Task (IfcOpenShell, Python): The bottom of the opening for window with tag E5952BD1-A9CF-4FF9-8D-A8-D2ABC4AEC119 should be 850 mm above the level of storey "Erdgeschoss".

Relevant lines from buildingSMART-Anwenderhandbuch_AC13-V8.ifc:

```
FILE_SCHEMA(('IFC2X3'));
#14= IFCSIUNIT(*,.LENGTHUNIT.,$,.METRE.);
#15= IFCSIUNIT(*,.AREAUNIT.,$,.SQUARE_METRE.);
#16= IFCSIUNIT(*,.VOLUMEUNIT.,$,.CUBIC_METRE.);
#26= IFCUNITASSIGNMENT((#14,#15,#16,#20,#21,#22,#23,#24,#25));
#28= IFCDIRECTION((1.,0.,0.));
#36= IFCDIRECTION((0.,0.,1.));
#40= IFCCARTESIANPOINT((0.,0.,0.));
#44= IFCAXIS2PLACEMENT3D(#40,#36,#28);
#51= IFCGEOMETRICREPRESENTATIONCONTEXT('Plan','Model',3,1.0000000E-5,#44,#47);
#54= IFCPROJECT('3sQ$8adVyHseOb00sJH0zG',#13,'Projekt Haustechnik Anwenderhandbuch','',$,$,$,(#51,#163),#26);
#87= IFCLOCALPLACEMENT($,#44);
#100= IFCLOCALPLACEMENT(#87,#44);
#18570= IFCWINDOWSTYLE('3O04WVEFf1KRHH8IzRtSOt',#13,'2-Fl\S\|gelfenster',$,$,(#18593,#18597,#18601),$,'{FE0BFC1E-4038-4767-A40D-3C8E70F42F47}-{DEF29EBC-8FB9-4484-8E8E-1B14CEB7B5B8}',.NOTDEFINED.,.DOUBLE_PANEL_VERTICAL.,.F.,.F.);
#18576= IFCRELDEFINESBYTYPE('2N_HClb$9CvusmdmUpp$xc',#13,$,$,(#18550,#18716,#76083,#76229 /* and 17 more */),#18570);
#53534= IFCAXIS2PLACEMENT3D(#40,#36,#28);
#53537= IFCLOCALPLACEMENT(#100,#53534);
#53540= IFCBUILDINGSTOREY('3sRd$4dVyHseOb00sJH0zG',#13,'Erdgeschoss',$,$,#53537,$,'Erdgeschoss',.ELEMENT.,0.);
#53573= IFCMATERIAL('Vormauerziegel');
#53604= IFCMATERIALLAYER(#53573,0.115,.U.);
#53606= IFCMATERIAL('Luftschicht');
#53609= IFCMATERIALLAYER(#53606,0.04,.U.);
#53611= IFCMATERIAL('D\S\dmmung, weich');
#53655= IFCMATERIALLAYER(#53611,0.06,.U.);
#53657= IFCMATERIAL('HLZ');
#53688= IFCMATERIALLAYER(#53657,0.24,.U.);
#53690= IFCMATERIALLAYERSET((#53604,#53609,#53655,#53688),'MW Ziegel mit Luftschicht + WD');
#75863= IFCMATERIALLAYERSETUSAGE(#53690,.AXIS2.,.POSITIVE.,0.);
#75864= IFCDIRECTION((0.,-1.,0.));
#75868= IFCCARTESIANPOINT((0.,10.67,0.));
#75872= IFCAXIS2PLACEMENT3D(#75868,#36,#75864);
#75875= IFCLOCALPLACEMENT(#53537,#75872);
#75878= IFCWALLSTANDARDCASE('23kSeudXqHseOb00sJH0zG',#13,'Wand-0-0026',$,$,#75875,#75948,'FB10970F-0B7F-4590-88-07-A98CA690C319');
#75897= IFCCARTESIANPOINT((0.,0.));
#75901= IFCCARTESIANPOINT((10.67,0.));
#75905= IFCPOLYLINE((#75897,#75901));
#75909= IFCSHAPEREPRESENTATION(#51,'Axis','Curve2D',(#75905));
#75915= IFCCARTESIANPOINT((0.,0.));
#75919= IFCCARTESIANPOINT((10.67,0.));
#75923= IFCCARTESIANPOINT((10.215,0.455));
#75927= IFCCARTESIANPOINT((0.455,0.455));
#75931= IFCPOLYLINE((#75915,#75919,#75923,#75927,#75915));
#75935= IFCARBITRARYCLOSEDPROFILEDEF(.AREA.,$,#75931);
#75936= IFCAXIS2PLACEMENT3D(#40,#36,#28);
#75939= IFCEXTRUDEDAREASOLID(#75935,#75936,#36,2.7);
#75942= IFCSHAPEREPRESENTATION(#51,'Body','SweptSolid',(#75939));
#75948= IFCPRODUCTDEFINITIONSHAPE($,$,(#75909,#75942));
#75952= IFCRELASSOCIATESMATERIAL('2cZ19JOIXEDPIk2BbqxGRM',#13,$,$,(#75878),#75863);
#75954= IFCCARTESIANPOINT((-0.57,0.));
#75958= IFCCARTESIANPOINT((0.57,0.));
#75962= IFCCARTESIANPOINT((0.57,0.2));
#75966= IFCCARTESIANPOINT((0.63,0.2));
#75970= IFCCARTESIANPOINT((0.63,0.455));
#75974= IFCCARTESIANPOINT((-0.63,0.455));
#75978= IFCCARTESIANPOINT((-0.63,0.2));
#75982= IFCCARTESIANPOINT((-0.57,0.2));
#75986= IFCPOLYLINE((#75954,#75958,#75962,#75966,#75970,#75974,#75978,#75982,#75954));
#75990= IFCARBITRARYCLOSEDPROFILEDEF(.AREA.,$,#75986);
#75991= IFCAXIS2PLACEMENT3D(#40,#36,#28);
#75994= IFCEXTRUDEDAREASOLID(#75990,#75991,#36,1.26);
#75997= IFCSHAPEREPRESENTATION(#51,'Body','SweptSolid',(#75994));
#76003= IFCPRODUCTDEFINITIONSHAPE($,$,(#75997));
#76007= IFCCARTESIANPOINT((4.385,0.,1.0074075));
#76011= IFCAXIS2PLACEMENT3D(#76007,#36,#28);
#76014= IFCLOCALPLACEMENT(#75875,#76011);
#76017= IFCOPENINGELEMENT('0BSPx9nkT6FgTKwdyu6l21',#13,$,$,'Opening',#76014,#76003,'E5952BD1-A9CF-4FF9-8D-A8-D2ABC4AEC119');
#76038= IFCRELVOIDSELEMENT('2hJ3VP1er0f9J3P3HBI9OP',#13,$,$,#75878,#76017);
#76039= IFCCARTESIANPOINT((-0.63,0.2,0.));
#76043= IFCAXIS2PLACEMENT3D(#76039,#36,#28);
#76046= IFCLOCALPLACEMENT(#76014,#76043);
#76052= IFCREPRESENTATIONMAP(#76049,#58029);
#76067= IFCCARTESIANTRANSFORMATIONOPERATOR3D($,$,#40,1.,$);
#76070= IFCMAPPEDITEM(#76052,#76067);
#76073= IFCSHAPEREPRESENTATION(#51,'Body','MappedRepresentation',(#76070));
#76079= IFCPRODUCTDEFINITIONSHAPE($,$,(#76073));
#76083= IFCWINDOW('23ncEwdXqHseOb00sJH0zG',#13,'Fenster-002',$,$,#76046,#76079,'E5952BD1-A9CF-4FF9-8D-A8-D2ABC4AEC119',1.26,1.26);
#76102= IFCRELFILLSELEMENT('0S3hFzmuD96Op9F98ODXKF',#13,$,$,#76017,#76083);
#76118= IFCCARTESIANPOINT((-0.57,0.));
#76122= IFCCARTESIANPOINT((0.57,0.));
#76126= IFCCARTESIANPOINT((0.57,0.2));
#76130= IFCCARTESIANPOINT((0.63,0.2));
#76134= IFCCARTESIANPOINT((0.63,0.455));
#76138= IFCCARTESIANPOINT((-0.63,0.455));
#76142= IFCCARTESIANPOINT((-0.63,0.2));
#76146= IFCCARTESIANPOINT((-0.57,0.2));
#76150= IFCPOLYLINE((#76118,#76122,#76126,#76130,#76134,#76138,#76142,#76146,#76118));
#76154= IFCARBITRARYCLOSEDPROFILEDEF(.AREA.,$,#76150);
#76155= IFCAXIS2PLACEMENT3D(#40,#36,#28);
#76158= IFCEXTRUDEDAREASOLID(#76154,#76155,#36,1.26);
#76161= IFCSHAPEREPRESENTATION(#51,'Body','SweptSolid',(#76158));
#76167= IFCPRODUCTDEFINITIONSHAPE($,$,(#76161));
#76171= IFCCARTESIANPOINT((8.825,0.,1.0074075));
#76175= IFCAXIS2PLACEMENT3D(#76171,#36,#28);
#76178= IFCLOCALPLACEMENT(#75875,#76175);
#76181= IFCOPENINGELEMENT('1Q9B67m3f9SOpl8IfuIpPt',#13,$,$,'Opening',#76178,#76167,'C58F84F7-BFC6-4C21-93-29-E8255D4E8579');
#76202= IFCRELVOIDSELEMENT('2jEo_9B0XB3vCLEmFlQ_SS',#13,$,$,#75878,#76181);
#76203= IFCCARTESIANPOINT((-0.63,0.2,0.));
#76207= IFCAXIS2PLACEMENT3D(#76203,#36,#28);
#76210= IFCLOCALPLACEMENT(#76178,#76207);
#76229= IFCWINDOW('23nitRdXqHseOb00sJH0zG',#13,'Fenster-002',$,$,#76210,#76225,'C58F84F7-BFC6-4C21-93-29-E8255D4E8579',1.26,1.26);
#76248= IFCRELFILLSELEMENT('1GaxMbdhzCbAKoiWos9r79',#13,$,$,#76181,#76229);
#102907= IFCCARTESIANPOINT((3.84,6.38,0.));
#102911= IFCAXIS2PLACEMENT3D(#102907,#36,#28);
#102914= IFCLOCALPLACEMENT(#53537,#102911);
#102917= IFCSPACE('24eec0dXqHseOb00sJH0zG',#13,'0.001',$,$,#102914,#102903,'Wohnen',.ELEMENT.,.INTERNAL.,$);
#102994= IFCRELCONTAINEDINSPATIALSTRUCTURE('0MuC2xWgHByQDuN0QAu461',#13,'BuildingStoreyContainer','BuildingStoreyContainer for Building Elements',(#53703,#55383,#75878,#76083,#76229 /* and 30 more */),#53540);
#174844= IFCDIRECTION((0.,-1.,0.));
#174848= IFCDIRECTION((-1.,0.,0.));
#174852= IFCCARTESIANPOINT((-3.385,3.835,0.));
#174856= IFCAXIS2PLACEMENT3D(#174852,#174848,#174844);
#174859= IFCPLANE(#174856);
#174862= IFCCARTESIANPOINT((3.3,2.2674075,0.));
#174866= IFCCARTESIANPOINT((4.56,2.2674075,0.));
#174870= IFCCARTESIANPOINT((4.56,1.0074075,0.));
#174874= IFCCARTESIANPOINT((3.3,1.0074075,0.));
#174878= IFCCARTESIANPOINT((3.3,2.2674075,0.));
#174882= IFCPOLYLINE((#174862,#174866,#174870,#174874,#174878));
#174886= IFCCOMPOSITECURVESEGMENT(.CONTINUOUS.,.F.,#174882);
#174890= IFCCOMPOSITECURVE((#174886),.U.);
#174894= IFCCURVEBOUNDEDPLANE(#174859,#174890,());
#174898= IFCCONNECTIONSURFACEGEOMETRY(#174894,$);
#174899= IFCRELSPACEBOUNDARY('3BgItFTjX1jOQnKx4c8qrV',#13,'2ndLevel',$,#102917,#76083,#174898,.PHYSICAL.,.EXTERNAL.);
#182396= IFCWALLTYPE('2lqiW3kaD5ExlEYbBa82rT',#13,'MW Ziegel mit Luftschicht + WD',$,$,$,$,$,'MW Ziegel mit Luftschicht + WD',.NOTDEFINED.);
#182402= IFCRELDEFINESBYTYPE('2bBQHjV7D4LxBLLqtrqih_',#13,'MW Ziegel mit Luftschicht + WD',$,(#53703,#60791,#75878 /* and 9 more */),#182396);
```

```python
import numpy as np
import ifcopenshell
import ifcopenshell.api.geometry
import ifcopenshell.geom
import ifcopenshell.util.element
import ifcopenshell.util.placement
import ifcopenshell.util.shape
import ifcopenshell.util.unit

model = ifcopenshell.open("buildingSMART-Anwenderhandbuch_AC13-V8.ifc")
unit_scale = ifcopenshell.util.unit.calculate_unit_scale(model)

window = model.by_guid("23ncEwdXqHseOb00sJH0zG")
opening = window.FillsVoids[0].RelatingOpeningElement
storey = ifcopenshell.util.element.get_container(window, ifc_class="IfcBuildingStorey")
level = ifcopenshell.util.placement.get_local_placement(storey.ObjectPlacement)[2, 3]

# The opening's origin need not be at the sill, so measure its lowest point.
shape = ifcopenshell.geom.create_shape(ifcopenshell.geom.settings(), opening)
bottom = ifcopenshell.util.shape.get_shape_bottom_elevation(shape, shape.geometry) / unit_scale
dz = level + 0.85 / unit_scale - bottom

shift = np.array([0.0, 0.0, dz])
# The window is placed relative to its opening, so it follows when the opening moves.
matrix = ifcopenshell.util.placement.get_local_placement(opening.ObjectPlacement)
matrix[:3, 3] += shift
ifcopenshell.api.geometry.edit_object_placement(
    model, product=opening, matrix=matrix, is_si=False, should_transform_children=True
)

# Space boundary surfaces are stored in each space's coordinates; move them too.
for rel in window.ProvidesBoundaries:
    if not rel.ConnectionGeometry:
        continue
    surface = rel.ConnectionGeometry.SurfaceOnRelatingElement.BasisSurface
    space_matrix = ifcopenshell.util.placement.get_local_placement(rel.RelatingSpace.ObjectPlacement)
    point = np.array(surface.Position.Location.Coordinates) + space_matrix[:3, :3].T @ shift
    surface.Position = model.createIfcAxis2Placement3D(
        model.createIfcCartesianPoint(point.tolist()), surface.Position.Axis, surface.Position.RefDirection
    )

print(f"moved by {dz * unit_scale:+.3f} m")

model.write("buildingSMART-Anwenderhandbuch_AC13-V8_rev.ifc")
```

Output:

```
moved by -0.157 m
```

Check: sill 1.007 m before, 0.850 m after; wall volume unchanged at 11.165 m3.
